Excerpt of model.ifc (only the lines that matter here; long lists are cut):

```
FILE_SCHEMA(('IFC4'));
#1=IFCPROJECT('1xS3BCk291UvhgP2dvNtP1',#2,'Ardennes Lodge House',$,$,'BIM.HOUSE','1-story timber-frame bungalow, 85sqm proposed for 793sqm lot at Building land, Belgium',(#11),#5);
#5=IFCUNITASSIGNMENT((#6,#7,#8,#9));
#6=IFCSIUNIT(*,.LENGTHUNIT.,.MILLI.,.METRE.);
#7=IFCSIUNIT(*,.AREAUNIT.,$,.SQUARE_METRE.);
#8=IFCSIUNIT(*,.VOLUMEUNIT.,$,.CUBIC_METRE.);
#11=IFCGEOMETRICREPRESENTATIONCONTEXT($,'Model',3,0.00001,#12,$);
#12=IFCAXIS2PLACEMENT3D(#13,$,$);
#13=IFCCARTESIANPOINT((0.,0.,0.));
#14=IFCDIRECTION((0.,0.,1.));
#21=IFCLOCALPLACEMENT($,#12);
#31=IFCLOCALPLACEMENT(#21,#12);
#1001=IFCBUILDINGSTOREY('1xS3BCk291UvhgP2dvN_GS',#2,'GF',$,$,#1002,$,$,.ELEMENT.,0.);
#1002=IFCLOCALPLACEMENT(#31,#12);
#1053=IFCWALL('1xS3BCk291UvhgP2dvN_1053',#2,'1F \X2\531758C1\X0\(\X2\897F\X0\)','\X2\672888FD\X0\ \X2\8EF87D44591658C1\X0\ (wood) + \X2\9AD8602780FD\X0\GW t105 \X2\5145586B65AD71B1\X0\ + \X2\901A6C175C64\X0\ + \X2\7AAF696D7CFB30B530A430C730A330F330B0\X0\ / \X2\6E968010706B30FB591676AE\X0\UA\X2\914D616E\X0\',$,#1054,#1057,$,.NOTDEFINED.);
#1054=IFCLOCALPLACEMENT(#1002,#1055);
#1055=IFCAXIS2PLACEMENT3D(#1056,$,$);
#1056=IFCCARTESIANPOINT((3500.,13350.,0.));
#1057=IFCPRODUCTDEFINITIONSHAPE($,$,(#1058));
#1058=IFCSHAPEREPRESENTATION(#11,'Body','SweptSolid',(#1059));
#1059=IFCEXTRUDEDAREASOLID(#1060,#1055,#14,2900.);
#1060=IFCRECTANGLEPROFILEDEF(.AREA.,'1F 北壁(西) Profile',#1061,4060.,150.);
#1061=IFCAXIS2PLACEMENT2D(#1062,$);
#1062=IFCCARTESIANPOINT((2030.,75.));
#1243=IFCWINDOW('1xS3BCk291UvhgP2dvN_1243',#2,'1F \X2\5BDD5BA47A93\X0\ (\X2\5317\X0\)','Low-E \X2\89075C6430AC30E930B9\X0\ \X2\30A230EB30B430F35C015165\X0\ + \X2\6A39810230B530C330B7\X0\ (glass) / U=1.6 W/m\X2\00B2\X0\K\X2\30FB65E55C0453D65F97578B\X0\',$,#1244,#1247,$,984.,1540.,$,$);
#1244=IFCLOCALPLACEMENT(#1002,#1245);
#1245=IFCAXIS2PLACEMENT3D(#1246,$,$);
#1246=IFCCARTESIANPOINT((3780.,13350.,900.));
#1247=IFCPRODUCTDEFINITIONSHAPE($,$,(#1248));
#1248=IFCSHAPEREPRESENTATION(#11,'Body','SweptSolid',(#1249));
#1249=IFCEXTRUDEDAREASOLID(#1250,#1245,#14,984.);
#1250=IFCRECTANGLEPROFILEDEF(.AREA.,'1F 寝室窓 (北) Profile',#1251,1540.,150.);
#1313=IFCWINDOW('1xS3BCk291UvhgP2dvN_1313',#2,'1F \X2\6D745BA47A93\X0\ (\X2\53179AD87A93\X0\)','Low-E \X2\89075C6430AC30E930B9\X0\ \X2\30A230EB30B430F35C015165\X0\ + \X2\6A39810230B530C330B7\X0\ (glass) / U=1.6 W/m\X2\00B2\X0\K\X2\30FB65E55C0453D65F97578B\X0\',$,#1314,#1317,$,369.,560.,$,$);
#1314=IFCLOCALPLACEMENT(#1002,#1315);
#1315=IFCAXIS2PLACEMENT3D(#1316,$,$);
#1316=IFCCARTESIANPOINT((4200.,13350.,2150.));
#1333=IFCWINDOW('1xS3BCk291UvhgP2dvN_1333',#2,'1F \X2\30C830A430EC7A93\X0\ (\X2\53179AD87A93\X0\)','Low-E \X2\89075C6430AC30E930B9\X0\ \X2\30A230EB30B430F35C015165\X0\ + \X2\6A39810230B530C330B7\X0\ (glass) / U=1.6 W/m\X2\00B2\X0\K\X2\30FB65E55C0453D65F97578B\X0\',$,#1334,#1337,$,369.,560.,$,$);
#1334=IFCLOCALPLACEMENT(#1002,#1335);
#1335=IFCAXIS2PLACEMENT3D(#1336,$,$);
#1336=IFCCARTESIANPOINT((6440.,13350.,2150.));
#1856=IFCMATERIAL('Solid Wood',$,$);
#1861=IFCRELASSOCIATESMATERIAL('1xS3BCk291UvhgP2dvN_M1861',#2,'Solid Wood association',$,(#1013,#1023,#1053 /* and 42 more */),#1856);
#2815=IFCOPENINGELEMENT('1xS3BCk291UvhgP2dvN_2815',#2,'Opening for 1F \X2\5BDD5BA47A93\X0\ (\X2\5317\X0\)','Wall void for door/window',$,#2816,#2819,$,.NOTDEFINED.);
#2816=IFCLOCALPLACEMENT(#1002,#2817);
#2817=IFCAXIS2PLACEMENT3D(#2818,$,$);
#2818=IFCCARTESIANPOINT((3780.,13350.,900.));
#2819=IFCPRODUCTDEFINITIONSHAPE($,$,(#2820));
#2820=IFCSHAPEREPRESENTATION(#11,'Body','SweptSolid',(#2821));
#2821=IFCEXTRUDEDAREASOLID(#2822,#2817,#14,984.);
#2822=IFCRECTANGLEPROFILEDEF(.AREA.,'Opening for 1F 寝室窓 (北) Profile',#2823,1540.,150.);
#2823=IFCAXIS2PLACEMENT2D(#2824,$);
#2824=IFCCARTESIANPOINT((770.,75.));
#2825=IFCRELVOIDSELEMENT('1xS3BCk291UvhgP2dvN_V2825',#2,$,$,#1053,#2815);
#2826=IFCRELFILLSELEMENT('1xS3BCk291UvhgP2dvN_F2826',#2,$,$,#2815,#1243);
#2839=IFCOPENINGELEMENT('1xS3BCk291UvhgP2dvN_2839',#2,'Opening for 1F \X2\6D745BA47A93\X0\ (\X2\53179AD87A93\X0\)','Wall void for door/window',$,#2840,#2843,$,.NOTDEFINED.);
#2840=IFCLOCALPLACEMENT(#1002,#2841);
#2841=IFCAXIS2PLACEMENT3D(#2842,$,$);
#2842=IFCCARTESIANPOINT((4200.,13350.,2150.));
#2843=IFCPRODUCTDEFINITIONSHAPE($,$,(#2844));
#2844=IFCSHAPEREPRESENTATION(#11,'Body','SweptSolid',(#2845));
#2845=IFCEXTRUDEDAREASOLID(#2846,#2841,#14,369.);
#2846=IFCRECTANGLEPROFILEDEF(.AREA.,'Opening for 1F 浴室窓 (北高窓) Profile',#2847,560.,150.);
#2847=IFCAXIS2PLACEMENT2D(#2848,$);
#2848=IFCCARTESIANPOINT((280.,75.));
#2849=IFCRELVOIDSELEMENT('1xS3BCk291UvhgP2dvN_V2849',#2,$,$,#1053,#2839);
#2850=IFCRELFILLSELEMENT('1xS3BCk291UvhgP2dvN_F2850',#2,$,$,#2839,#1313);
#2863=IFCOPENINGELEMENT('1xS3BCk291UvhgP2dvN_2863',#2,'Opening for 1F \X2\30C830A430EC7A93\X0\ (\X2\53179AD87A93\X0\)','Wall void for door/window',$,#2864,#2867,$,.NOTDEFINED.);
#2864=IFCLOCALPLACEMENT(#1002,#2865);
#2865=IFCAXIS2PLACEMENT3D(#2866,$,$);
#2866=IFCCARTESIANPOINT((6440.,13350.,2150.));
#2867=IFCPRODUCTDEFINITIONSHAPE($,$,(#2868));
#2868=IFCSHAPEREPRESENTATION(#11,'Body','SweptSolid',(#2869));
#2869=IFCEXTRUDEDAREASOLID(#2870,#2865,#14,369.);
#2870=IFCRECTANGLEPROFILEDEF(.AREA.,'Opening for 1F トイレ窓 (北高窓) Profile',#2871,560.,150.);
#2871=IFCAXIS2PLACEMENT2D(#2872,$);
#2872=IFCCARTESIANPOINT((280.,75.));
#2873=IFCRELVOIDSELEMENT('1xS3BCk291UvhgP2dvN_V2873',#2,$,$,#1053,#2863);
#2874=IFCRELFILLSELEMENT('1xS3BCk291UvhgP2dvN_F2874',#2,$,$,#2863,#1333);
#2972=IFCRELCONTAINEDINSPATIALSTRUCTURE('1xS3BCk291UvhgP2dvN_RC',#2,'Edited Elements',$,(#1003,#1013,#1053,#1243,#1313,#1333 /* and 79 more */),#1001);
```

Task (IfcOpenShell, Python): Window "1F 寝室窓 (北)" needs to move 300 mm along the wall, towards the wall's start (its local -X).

```python
import ifcopenshell
import ifcopenshell.api.geometry
import ifcopenshell.util.placement

model = ifcopenshell.open("model.ifc")

window = model.by_id(1243)
opening = window.FillsVoids[0].RelatingOpeningElement
wall = opening.VoidsElements[0].RelatingBuildingElement

wall_matrix = ifcopenshell.util.placement.get_local_placement(wall.ObjectPlacement)
shift = wall_matrix[:3, 0] * -300.0
before = ifcopenshell.util.placement.get_local_placement(window.ObjectPlacement)[:3, 3].copy()

# The window is not placed relative to its opening, so move both.
for product in (opening, window):
    matrix = ifcopenshell.util.placement.get_local_placement(product.ObjectPlacement)
    matrix[:3, 3] += shift
    ifcopenshell.api.geometry.edit_object_placement(model, product=product, matrix=matrix, is_si=False)

after = ifcopenshell.util.placement.get_local_placement(window.ObjectPlacement)[:3, 3]
print("window moved by", (after - before).round(3) + 0.0)

model.write("model-out.ifc")
```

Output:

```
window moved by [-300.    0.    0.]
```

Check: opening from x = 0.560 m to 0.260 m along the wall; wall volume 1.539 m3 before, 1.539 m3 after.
